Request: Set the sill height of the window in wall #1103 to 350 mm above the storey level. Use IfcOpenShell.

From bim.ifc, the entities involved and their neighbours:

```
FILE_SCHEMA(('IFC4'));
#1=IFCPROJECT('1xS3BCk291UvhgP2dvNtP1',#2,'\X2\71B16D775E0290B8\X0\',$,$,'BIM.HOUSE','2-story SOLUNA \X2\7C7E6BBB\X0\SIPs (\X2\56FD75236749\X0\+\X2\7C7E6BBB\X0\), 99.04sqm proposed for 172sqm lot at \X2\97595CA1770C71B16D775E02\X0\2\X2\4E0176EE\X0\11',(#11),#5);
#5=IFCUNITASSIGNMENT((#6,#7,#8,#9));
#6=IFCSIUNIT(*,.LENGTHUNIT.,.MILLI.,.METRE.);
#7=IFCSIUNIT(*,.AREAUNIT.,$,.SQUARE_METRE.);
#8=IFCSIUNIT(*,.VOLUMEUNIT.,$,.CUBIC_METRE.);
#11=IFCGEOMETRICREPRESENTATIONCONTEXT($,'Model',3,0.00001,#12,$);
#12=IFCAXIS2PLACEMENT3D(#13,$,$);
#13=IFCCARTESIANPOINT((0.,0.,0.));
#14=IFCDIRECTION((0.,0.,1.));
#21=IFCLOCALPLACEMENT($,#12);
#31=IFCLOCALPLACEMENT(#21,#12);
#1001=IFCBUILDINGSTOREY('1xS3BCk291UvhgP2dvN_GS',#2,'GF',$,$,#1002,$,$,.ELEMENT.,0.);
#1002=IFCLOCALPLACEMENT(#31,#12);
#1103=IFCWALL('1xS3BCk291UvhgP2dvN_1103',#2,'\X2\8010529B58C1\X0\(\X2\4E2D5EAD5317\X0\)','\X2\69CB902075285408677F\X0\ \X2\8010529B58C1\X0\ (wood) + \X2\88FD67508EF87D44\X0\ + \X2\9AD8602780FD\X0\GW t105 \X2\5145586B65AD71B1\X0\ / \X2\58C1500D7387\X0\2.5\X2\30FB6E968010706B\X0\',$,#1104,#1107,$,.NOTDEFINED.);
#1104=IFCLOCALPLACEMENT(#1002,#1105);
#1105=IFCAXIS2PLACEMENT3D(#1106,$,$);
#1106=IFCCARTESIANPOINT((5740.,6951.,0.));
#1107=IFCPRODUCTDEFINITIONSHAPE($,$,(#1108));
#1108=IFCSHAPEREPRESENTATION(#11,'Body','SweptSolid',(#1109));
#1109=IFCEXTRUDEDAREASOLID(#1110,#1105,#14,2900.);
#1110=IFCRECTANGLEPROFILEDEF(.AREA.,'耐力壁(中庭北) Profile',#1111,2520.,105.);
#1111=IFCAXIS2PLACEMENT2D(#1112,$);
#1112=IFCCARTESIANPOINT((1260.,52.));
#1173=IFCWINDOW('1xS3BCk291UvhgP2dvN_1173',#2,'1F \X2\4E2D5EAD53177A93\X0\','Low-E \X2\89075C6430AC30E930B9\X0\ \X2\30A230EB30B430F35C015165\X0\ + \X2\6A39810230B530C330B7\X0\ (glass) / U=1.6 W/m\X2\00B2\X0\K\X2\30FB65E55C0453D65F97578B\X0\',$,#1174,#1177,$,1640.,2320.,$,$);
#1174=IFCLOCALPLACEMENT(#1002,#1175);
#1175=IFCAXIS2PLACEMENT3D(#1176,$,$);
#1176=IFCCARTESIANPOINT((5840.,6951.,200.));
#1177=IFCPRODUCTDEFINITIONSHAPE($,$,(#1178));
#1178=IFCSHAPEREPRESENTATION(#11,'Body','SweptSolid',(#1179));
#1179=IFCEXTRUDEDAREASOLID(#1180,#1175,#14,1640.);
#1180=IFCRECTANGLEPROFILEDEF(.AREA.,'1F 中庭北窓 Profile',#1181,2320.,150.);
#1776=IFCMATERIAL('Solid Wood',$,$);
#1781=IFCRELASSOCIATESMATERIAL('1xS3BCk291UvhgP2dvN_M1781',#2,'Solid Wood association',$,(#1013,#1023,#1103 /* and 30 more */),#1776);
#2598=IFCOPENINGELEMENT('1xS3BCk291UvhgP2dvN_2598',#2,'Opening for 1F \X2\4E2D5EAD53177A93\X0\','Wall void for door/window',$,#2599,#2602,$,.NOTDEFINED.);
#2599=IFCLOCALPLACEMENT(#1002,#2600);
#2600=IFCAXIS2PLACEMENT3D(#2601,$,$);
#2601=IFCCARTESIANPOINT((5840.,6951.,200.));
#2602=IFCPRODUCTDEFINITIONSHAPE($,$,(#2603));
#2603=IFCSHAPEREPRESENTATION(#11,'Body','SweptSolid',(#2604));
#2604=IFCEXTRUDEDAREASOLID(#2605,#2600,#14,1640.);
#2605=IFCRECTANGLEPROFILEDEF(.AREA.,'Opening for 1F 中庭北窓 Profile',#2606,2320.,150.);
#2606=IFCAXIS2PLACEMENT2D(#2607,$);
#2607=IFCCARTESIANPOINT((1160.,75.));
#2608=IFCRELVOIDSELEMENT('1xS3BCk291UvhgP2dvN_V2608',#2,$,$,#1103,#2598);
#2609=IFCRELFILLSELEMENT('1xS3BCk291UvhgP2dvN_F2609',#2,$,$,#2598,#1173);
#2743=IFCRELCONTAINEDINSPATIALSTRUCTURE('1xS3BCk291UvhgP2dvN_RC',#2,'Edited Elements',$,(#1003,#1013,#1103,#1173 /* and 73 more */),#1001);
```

```python
import numpy as np
import ifcopenshell
import ifcopenshell.api.geometry
import ifcopenshell.geom
import ifcopenshell.util.element
import ifcopenshell.util.placement
import ifcopenshell.util.shape
import ifcopenshell.util.unit

model = ifcopenshell.open("bim.ifc")
unit_scale = ifcopenshell.util.unit.calculate_unit_scale(model)

window = model.by_id(1173)
opening = window.FillsVoids[0].RelatingOpeningElement
storey = ifcopenshell.util.element.get_container(window, ifc_class="IfcBuildingStorey")
level = ifcopenshell.util.placement.get_local_placement(storey.ObjectPlacement)[2, 3]

# The opening's origin need not be at the sill, so measure its lowest point.
shape = ifcopenshell.geom.create_shape(ifcopenshell.geom.settings(), opening)
bottom = ifcopenshell.util.shape.get_shape_bottom_elevation(shape, shape.geometry) / unit_scale
dz = level + 0.35 / unit_scale - bottom

shift = np.array([0.0, 0.0, dz])
# The window is not placed relative to its opening, so move both.
for product in (opening, window):
    matrix = ifcopenshell.util.placement.get_local_placement(product.ObjectPlacement)
    matrix[:3, 3] += shift
    ifcopenshell.api.geometry.edit_object_placement(model, product=product, matrix=matrix, is_si=False)

print(f"moved by {dz * unit_scale:+.3f} m")

model.write("bim_updated.ifc")
```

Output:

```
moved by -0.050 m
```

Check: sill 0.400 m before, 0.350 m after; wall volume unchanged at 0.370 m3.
